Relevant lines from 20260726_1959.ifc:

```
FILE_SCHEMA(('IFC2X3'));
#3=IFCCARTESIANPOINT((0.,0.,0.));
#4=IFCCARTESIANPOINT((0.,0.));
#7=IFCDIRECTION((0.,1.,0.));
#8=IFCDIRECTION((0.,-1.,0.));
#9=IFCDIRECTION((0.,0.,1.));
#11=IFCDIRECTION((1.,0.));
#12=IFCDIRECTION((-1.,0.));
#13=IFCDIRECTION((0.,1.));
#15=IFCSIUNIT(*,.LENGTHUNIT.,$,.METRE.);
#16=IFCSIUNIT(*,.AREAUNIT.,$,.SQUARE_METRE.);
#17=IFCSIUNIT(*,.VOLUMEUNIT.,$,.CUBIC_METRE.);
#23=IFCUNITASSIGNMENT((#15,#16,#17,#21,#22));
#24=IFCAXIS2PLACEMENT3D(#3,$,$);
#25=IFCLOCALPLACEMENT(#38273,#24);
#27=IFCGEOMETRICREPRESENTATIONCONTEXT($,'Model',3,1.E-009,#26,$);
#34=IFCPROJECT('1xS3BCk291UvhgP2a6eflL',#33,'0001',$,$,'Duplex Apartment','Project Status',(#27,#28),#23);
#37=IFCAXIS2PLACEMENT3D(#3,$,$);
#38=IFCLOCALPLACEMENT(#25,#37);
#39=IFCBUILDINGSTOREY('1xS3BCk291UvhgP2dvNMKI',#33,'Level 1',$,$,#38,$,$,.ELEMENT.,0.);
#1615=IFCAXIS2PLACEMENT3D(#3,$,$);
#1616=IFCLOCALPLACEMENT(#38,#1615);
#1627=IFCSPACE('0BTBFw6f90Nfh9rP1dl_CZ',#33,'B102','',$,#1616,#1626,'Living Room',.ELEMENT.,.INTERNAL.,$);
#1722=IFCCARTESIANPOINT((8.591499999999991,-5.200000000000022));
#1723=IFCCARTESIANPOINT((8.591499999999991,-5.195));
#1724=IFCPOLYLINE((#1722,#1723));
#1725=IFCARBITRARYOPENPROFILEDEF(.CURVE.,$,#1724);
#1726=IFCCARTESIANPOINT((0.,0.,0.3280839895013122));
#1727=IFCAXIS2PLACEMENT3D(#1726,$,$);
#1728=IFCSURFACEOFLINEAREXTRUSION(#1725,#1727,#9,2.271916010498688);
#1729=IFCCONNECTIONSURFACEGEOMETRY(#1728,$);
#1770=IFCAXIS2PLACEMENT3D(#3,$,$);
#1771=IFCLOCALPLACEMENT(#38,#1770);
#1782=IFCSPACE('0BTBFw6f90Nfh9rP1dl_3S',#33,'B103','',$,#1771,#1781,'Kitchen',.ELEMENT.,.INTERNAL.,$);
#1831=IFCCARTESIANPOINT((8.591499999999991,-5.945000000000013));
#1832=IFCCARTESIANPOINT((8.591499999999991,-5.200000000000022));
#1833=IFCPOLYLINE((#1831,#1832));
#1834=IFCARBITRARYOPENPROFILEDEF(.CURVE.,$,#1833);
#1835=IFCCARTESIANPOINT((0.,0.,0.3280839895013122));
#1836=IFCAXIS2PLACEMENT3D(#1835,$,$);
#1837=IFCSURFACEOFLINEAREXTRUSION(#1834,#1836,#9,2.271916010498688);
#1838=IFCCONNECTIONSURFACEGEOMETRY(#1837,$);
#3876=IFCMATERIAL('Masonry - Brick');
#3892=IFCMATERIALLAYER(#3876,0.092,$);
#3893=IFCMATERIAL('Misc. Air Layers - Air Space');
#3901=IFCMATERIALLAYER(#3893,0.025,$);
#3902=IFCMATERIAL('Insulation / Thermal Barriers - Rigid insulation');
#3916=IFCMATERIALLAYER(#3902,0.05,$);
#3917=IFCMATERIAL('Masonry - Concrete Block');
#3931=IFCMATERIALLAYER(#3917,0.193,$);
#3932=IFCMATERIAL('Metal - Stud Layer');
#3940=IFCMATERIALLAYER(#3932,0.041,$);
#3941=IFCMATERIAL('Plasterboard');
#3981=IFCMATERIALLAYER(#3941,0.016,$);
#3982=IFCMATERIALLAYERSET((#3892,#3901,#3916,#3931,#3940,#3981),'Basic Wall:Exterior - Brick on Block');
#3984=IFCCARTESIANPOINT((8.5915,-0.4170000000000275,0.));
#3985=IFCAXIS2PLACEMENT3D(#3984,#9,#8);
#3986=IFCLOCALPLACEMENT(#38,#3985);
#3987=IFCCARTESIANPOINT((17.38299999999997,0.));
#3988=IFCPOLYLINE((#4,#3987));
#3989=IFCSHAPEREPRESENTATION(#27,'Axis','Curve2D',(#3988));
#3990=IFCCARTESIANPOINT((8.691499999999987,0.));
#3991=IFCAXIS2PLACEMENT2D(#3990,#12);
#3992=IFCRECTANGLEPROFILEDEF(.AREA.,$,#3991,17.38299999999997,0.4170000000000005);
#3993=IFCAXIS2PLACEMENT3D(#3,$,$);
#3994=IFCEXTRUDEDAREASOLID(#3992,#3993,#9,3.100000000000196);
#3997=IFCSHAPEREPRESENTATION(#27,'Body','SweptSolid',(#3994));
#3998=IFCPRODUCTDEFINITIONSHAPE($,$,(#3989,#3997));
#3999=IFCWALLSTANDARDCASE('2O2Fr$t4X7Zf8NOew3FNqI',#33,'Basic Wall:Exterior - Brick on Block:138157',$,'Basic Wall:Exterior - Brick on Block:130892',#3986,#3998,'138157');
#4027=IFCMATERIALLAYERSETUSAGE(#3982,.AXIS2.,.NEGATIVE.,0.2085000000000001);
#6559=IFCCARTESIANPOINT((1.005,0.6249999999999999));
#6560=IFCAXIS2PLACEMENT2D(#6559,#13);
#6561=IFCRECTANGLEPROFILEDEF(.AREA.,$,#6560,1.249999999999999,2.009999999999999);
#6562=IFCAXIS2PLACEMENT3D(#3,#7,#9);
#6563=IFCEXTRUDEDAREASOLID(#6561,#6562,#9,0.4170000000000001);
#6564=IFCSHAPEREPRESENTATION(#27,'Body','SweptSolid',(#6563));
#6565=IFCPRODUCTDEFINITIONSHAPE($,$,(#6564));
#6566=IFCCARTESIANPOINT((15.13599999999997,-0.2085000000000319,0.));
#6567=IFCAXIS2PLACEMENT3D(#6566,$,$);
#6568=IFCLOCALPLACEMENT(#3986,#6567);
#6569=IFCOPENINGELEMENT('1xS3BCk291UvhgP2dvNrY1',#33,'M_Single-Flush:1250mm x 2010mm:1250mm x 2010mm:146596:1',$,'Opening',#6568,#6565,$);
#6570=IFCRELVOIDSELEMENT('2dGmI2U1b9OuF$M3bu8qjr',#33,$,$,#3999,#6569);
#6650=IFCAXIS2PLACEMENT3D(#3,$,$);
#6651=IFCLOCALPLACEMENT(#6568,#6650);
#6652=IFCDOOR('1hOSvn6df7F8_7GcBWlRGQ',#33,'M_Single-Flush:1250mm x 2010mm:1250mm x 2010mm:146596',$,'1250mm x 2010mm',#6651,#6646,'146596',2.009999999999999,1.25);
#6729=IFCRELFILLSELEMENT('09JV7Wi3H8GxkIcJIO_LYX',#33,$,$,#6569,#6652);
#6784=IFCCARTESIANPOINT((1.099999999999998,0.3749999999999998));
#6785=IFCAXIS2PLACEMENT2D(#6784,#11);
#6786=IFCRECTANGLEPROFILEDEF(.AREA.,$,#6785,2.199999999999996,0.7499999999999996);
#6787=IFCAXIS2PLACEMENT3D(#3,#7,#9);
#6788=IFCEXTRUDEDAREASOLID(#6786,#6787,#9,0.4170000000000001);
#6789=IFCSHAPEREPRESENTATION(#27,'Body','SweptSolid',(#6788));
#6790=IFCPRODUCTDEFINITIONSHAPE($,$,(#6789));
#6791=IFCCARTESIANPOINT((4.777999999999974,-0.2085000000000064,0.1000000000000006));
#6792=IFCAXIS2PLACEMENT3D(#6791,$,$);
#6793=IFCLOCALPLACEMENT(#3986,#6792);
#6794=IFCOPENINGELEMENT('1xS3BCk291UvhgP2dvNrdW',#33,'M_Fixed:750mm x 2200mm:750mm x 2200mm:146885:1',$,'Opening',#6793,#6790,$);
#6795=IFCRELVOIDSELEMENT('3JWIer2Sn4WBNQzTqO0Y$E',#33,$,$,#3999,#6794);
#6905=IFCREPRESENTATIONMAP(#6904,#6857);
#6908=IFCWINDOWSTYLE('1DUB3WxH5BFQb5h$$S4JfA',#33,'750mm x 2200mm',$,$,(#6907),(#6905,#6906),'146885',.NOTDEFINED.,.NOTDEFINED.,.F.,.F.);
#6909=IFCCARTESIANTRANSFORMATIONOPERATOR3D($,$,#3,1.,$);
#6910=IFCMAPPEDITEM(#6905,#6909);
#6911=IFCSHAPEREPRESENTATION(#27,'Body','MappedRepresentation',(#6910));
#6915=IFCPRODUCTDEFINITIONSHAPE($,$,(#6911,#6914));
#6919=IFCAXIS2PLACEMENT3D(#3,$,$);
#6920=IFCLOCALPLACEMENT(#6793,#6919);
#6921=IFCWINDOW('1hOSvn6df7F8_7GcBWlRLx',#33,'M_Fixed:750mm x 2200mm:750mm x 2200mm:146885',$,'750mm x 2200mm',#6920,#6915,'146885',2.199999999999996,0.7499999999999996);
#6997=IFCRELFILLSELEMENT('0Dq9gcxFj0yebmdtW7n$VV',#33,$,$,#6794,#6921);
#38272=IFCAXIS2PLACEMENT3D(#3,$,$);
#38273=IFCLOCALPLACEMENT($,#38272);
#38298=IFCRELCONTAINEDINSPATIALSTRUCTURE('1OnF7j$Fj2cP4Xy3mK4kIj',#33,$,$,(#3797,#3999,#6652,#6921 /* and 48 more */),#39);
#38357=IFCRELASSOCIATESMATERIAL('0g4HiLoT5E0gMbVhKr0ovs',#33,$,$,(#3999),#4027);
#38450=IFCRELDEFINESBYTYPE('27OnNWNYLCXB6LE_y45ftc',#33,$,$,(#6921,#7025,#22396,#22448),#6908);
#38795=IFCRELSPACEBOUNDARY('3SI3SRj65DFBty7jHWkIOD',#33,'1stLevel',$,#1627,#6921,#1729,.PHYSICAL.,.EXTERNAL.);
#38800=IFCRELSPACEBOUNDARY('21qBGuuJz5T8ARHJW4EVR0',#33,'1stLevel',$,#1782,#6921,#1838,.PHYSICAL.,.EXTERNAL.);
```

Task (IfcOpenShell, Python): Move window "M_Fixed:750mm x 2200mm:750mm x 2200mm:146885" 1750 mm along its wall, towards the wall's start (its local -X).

```python
import numpy as np
import ifcopenshell
import ifcopenshell.api.geometry
import ifcopenshell.util.placement
import ifcopenshell.util.unit

model = ifcopenshell.open("20260726_1959.ifc")
unit_scale = ifcopenshell.util.unit.calculate_unit_scale(model)

window = model.by_guid("1hOSvn6df7F8_7GcBWlRLx")
opening = window.FillsVoids[0].RelatingOpeningElement
wall = opening.VoidsElements[0].RelatingBuildingElement

wall_matrix = ifcopenshell.util.placement.get_local_placement(wall.ObjectPlacement)
shift = wall_matrix[:3, 0] * -1.75 / unit_scale
before = ifcopenshell.util.placement.get_local_placement(window.ObjectPlacement)[:3, 3].copy()

# The window is placed relative to its opening, so it follows when the opening moves.
matrix = ifcopenshell.util.placement.get_local_placement(opening.ObjectPlacement)
matrix[:3, 3] += shift
ifcopenshell.api.geometry.edit_object_placement(
    model, product=opening, matrix=matrix, is_si=False, should_transform_children=True
)

# Space boundary surfaces are stored in each space's coordinates; move them too.
for rel in window.ProvidesBoundaries:
    if not rel.ConnectionGeometry:
        continue
    surface = rel.ConnectionGeometry.SurfaceOnRelatingElement
    space_matrix = ifcopenshell.util.placement.get_local_placement(rel.RelatingSpace.ObjectPlacement)
    point = np.array(surface.Position.Location.Coordinates) + space_matrix[:3, :3].T @ shift
    surface.Position = model.createIfcAxis2Placement3D(
        model.createIfcCartesianPoint(point.tolist()), surface.Position.Axis, surface.Position.RefDirection
    )

after = ifcopenshell.util.placement.get_local_placement(window.ObjectPlacement)[:3, 3]
print("window moved by", (after - before).round(3) + 0.0)

model.write("20260726_1959_rev.ifc")
```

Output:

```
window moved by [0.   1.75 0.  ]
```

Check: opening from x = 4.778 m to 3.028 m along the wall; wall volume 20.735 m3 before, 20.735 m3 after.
